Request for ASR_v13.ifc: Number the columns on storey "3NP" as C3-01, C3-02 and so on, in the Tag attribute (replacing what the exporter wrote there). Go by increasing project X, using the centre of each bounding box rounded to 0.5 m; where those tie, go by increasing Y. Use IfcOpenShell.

First a look at what the model holds.

```python
import ifcopenshell
import ifcopenshell.util.element
import ifcopenshell.util.placement

model = ifcopenshell.open("ASR_v13.ifc")
print(model.schema)
storey = next(s for s in model.by_type("IfcBuildingStorey") if s.Name == "3NP")
columns = [e for e in ifcopenshell.util.element.get_decomposition(storey) if e.is_a("IfcColumn")]
for e in sorted(columns, key=lambda e: e.id()):
    origin = ifcopenshell.util.placement.get_local_placement(e.ObjectPlacement)[:3, 3]
    print(e.id(), e.Tag, e.Name, origin.round(2) + 0.0, sep=" | ")
```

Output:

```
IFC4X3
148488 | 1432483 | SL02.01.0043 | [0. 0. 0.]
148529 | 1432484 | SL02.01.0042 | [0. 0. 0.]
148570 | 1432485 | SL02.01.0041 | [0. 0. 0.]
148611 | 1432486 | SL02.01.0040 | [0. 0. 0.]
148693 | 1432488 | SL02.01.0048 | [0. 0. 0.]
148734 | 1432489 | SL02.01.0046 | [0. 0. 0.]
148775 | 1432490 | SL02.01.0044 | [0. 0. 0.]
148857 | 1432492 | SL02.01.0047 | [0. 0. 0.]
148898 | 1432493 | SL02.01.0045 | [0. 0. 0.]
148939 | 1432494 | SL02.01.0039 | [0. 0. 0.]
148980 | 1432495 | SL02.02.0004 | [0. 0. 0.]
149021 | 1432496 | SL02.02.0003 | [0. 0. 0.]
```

```python
import ifcopenshell
import ifcopenshell.geom
import ifcopenshell.util.element
import ifcopenshell.util.shape

model = ifcopenshell.open("ASR_v13.ifc")
settings = ifcopenshell.geom.settings()
settings.set("use-world-coords", True)


def centre(element):
    shape = ifcopenshell.geom.create_shape(settings, element)
    return ifcopenshell.util.shape.get_bbox_centroid(shape.geometry)


storey = next(s for s in model.by_type("IfcBuildingStorey") if s.Name == "3NP")
columns = [e for e in ifcopenshell.util.element.get_decomposition(storey) if e.is_a("IfcColumn")]

# Insertion points can sit at a corner or the storey origin, so sort by the geometry (in metres).
centres = {e: centre(e) for e in columns}
columns.sort(key=lambda e: (round(centres[e][0] / 0.5), centres[e][1]))

for i, e in enumerate(columns, start=1):
    number = f"C3-{i:02d}"
    e.Tag = number
    print(e.id(), number)

model.write("ASR_v13_updated.ifc")
```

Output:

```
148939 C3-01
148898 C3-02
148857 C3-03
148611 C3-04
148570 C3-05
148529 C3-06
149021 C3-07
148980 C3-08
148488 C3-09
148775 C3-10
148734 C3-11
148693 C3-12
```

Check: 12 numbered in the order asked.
